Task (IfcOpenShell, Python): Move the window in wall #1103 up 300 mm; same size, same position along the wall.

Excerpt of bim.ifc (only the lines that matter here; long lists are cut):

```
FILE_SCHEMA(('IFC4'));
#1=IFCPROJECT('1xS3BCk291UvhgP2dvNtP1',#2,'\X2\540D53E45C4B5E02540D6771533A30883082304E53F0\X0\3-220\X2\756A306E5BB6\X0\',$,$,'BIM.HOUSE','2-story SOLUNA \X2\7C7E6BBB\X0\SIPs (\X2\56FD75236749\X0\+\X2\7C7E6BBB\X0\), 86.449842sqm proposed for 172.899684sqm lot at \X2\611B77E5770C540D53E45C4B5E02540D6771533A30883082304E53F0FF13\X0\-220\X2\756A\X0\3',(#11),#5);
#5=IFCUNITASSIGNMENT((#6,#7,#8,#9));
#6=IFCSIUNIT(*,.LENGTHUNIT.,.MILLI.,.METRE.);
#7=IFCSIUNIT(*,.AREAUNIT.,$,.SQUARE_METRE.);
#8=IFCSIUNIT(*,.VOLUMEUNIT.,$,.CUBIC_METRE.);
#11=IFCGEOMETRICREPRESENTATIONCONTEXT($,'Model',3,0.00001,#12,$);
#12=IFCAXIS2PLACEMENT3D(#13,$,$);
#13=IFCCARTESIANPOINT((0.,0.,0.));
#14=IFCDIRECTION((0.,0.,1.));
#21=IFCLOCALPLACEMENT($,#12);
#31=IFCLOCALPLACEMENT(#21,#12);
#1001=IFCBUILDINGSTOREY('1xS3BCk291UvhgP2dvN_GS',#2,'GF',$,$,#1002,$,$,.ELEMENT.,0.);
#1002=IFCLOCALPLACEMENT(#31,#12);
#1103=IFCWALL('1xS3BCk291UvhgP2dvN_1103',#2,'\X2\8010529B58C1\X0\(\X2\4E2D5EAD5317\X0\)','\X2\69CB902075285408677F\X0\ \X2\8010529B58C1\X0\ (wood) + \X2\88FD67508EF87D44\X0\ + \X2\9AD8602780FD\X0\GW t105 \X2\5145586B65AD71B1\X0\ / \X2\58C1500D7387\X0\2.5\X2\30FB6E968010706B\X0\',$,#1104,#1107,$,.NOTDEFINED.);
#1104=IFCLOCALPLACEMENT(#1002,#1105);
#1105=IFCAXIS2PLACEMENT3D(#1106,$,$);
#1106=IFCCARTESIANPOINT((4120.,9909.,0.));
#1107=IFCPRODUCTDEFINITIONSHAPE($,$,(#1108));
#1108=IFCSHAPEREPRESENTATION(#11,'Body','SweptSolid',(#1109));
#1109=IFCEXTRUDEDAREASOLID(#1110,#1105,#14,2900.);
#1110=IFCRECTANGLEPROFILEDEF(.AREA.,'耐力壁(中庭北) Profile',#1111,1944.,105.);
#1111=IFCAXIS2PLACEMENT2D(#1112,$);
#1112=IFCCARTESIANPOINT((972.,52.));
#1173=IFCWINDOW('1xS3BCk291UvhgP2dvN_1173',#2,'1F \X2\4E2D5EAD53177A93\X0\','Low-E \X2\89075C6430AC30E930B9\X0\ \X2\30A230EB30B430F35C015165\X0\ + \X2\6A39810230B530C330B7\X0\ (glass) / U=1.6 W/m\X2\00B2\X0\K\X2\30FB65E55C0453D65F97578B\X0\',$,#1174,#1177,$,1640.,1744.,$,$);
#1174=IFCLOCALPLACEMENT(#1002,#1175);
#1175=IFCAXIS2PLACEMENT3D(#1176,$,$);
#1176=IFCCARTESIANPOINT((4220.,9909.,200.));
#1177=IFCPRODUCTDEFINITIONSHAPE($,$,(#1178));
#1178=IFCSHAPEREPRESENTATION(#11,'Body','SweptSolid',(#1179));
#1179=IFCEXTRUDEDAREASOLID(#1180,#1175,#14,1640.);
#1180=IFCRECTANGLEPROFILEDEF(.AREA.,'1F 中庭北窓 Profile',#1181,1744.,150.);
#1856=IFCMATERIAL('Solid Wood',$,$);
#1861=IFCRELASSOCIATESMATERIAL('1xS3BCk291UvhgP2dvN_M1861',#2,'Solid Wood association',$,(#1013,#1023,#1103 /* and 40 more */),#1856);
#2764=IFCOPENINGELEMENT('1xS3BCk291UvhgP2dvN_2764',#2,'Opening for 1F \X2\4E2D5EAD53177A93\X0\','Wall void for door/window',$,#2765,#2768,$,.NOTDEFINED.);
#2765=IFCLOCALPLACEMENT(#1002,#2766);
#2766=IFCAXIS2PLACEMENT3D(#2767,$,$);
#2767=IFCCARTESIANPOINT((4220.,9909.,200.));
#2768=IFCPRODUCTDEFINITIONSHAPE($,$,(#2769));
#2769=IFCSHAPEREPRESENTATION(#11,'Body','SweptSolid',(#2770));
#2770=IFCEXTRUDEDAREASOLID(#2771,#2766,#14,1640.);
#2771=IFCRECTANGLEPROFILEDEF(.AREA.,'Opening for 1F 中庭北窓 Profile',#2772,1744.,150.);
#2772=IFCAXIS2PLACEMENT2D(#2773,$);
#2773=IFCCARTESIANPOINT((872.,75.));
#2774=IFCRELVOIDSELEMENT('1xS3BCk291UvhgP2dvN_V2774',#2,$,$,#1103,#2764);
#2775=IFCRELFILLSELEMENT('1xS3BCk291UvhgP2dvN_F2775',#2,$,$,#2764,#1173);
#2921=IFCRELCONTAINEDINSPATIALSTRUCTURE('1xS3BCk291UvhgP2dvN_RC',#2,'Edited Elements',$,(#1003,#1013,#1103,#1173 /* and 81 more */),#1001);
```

```python
import numpy as np
import ifcopenshell
import ifcopenshell.api.geometry
import ifcopenshell.util.placement
import ifcopenshell.util.unit

model = ifcopenshell.open("bim.ifc")
unit_scale = ifcopenshell.util.unit.calculate_unit_scale(model)

window = model.by_guid("1xS3BCk291UvhgP2dvN_1173")
opening = window.FillsVoids[0].RelatingOpeningElement
dz = 300.0

shift = np.array([0.0, 0.0, dz])
# The window is not placed relative to its opening, so move both.
for product in (opening, window):
    matrix = ifcopenshell.util.placement.get_local_placement(product.ObjectPlacement)
    matrix[:3, 3] += shift
    ifcopenshell.api.geometry.edit_object_placement(model, product=product, matrix=matrix, is_si=False)

print(f"moved by {dz * unit_scale:+.3f} m")

model.write("bim_edited.ifc")
```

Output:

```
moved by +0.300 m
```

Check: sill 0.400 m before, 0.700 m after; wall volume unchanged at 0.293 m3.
